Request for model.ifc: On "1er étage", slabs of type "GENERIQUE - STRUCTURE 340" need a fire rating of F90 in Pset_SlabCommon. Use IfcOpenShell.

First a look at what the model holds.

```python
import ifcopenshell
import ifcopenshell.util.element

model = ifcopenshell.open("model.ifc")
print(model.schema)
storey = next(s for s in model.by_type("IfcBuildingStorey") if s.Name == "1er étage")
slabs = [e for e in ifcopenshell.util.element.get_decomposition(storey) if e.is_a("IfcSlab")]
seen = {}
for e in slabs:
    element_type = ifcopenshell.util.element.get_type(e)
    key = (element_type.Name if element_type != e and element_type else None, ifcopenshell.util.element.get_pset(e, "Pset_SlabCommon", "FireRating"))
    seen[key] = seen.get(key, 0) + 1
for (name, value), count in sorted(seen.items(), key=str):
    print(count, "x", name, "|", value)
```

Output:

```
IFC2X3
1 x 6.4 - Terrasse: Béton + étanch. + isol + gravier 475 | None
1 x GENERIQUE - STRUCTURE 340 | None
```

```python
import ifcopenshell
import ifcopenshell.api.pset
import ifcopenshell.util.element

model = ifcopenshell.open("model.ifc")

storey = next(s for s in model.by_type("IfcBuildingStorey") if s.Name == "1er étage")
slabs = [e for e in ifcopenshell.util.element.get_decomposition(storey) if e.is_a("IfcSlab")]

count = 0
for e in slabs:
    element_type = ifcopenshell.util.element.get_type(e)
    if element_type in (None, e) or element_type.Name != "GENERIQUE - STRUCTURE 340":
        continue
    # add_pset returns the element's existing set when there is one.
    pset = ifcopenshell.api.pset.add_pset(model, product=e, name="Pset_SlabCommon")
    ifcopenshell.api.pset.edit_pset(model, pset=pset, properties={"FireRating": "F90"})
    count += 1

print(count, "slabs updated")

model.write("model_updated.ifc")
```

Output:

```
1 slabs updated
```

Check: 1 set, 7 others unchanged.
